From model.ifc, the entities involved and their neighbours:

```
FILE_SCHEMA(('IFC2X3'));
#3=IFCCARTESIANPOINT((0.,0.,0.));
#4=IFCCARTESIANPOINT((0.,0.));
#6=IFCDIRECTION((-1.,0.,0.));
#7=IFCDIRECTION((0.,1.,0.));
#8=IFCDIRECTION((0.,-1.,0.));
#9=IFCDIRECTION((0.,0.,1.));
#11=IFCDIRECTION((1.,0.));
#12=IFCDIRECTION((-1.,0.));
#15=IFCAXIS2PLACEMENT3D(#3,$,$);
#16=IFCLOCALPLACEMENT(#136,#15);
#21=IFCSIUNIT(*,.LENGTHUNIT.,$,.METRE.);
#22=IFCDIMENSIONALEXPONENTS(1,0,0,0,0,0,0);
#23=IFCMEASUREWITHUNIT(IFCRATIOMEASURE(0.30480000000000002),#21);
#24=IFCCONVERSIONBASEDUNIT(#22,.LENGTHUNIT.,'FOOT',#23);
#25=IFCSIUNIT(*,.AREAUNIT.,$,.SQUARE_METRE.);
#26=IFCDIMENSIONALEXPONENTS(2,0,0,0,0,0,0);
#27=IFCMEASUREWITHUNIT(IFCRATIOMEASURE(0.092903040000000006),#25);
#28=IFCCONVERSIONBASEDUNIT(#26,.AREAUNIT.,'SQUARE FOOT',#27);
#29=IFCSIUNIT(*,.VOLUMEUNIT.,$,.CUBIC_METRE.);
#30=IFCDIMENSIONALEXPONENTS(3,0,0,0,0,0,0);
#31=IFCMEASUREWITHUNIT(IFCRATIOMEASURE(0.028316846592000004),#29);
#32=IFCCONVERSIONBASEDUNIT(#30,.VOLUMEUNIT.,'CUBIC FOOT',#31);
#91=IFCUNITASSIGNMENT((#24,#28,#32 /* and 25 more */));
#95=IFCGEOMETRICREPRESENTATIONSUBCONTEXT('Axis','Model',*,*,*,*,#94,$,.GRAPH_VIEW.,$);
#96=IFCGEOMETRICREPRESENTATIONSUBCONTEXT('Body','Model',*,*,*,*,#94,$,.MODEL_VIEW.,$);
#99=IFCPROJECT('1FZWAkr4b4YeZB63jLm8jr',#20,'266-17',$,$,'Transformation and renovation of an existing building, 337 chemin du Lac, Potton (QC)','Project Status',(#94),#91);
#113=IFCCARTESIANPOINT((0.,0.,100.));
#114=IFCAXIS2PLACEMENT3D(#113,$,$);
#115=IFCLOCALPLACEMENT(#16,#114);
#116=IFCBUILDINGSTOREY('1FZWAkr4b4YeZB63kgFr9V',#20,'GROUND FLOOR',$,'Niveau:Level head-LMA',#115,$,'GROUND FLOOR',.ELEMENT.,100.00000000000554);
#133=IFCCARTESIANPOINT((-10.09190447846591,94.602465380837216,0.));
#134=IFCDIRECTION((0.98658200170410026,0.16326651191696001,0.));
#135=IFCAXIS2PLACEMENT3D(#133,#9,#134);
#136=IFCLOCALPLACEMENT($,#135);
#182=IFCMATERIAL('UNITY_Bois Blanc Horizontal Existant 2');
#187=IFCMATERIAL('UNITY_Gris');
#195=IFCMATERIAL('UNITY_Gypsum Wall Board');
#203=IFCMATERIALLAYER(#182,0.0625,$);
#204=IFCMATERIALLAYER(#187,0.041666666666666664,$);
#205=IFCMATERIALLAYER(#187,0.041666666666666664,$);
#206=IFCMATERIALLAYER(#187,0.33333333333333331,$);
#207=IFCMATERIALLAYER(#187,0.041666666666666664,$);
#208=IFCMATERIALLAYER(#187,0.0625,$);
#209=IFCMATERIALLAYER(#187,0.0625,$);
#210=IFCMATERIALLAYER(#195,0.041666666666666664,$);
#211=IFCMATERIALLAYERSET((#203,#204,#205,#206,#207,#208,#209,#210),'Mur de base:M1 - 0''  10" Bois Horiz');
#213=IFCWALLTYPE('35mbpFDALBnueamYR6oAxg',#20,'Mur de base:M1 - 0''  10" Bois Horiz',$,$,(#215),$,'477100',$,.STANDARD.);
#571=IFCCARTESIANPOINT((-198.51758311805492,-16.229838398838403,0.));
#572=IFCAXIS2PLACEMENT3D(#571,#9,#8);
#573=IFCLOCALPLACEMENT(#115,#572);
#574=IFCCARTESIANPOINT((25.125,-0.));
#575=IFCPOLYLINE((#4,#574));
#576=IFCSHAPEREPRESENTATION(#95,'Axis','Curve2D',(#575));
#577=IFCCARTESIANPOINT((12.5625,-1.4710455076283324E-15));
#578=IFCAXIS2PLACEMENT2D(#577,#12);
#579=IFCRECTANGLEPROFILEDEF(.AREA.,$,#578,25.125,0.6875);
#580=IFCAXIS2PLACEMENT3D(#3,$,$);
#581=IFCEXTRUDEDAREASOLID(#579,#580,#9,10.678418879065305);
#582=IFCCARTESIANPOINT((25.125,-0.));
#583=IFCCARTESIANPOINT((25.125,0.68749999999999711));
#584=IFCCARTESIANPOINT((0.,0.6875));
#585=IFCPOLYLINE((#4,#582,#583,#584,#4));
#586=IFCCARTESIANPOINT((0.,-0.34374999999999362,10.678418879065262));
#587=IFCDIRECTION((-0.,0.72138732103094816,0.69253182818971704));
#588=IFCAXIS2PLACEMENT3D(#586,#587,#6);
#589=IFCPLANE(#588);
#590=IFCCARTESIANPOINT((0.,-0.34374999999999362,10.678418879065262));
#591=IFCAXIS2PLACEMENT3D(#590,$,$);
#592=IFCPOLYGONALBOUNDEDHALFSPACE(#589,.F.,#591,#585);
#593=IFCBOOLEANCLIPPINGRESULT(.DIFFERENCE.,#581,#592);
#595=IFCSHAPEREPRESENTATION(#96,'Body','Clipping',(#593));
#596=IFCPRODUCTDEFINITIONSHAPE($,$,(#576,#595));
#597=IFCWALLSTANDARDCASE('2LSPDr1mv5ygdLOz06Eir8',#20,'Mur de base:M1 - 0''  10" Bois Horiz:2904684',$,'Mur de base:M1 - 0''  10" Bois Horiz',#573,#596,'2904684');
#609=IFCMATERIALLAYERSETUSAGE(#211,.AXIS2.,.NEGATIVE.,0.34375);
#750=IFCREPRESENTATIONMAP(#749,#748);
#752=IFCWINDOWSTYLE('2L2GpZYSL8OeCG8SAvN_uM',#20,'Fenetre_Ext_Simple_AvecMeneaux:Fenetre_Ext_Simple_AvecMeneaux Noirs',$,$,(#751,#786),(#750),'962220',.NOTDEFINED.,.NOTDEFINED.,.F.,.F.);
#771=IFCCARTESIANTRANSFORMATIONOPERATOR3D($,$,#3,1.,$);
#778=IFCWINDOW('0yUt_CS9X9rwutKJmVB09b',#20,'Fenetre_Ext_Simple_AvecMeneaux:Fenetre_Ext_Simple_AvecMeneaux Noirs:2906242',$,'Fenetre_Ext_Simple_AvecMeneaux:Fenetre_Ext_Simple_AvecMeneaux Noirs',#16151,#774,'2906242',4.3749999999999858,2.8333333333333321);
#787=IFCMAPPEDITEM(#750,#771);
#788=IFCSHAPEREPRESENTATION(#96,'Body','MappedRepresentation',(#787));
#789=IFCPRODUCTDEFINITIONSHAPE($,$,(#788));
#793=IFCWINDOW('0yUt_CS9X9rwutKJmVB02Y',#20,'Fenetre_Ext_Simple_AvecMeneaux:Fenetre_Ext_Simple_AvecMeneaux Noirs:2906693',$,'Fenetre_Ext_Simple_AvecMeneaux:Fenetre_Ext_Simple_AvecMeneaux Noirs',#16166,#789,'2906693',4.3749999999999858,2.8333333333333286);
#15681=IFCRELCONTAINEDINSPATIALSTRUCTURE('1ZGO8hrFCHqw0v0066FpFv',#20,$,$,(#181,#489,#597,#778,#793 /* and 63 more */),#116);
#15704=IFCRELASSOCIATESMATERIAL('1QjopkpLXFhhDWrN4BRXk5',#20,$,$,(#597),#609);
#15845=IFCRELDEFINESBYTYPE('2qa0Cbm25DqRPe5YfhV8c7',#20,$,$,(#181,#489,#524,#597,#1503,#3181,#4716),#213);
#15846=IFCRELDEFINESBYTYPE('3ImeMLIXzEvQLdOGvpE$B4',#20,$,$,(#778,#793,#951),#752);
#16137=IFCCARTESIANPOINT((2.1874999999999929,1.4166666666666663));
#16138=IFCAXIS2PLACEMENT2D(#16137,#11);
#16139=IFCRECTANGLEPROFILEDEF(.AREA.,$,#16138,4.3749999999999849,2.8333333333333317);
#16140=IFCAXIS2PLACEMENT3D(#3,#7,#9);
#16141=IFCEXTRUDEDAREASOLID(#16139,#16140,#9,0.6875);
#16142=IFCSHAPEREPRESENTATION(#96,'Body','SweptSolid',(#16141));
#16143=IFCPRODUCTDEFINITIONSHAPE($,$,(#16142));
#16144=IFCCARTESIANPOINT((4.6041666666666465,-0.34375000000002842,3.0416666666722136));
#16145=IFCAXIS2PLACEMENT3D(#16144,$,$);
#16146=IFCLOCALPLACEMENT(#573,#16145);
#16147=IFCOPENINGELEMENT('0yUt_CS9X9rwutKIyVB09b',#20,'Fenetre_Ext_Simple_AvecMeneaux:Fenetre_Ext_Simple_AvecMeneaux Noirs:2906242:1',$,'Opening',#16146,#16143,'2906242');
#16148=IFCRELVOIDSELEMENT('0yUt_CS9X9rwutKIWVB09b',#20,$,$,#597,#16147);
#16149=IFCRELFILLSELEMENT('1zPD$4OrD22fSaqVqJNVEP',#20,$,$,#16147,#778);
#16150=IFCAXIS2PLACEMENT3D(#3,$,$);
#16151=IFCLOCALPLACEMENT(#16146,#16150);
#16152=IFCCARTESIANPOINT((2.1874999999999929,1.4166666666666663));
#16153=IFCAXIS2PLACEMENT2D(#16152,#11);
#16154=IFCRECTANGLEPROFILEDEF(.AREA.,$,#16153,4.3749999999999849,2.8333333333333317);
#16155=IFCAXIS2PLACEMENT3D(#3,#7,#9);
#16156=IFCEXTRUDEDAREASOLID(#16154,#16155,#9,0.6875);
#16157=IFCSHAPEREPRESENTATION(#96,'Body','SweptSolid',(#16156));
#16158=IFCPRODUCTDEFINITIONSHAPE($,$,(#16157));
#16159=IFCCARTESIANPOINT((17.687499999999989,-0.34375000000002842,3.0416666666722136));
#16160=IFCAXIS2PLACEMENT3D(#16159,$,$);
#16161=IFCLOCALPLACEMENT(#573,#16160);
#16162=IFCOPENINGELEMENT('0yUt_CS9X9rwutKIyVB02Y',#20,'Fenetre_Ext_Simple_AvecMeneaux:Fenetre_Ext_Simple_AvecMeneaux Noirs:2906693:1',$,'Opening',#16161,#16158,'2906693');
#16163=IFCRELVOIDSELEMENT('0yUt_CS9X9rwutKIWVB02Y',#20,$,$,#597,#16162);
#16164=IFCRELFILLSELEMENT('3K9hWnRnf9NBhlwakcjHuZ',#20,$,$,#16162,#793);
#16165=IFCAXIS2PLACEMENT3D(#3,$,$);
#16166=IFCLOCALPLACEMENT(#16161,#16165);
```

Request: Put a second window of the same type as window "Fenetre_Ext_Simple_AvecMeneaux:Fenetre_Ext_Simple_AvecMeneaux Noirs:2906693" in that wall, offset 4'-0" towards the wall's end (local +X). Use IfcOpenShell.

```python
import ifcopenshell
import ifcopenshell.api.feature
import ifcopenshell.api.geometry
import ifcopenshell.api.root
import ifcopenshell.geom
import ifcopenshell.util.element
import ifcopenshell.util.placement
import ifcopenshell.util.shape
import ifcopenshell.util.unit

model = ifcopenshell.open("model.ifc")
unit_scale = ifcopenshell.util.unit.calculate_unit_scale(model)
settings = ifcopenshell.geom.settings()


def volume(element):
    """Net volume in cubic metres, openings subtracted."""
    shape = ifcopenshell.geom.create_shape(settings, element)
    return ifcopenshell.util.shape.get_volume(shape.geometry)


def reuse_history(source, copy):
    """copy_class also copies each property set's owner history, people and application; keep the originals."""
    for rel in copy.IsDefinedBy:
        if rel.is_a("IfcRelDefinesByProperties") and (history := rel.RelatingPropertyDefinition.OwnerHistory):
            rel.RelatingPropertyDefinition.OwnerHistory = source.OwnerHistory
            ifcopenshell.util.element.remove_deep2(model, history)


window = model.by_guid("0yUt_CS9X9rwutKJmVB02Y")
opening = window.FillsVoids[0].RelatingOpeningElement
wall = opening.VoidsElements[0].RelatingBuildingElement
before = volume(wall)
shift = ifcopenshell.util.placement.get_local_placement(wall.ObjectPlacement)[:3, 0] * 48 * 0.0254 / unit_scale

# copy_class copies the void relationship, type, container and properties, but no geometry.
new_opening = ifcopenshell.api.root.copy_class(model, product=opening)
new_opening.Representation = ifcopenshell.util.element.copy_deep(
    model, opening.Representation, exclude=["IfcGeometricRepresentationContext", "IfcRepresentationMap"]
)
new_opening.Name = "Fenetre_Ext_Simple_AvecMeneaux:Fenetre_Ext_Simple_AvecMeneaux Noirs"
new_opening.Tag = None
new_window = ifcopenshell.api.root.copy_class(model, product=window)
new_window.Representation = ifcopenshell.util.element.copy_deep(
    model, window.Representation, exclude=["IfcGeometricRepresentationContext", "IfcRepresentationMap"]
)
new_window.Name = "Fenetre_Ext_Simple_AvecMeneaux:Fenetre_Ext_Simple_AvecMeneaux Noirs"
new_window.Tag = None
reuse_history(window, new_window)
fills = ifcopenshell.api.feature.add_filling(model, opening=new_opening, element=new_window)
fills.OwnerHistory = new_window.OwnerHistory  # required in IFC2X3

for old, new in ((opening, new_opening), (window, new_window)):
    matrix = ifcopenshell.util.placement.get_local_placement(old.ObjectPlacement)
    matrix[:3, 3] += shift
    ifcopenshell.api.geometry.edit_object_placement(model, product=new, matrix=matrix, is_si=False)

after = volume(wall)

print(f"wall volume {before:.3f} -> {after:.3f} m3")

model.write("model_edited.ifc")
```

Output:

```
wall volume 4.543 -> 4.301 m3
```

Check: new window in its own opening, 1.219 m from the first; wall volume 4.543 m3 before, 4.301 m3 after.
